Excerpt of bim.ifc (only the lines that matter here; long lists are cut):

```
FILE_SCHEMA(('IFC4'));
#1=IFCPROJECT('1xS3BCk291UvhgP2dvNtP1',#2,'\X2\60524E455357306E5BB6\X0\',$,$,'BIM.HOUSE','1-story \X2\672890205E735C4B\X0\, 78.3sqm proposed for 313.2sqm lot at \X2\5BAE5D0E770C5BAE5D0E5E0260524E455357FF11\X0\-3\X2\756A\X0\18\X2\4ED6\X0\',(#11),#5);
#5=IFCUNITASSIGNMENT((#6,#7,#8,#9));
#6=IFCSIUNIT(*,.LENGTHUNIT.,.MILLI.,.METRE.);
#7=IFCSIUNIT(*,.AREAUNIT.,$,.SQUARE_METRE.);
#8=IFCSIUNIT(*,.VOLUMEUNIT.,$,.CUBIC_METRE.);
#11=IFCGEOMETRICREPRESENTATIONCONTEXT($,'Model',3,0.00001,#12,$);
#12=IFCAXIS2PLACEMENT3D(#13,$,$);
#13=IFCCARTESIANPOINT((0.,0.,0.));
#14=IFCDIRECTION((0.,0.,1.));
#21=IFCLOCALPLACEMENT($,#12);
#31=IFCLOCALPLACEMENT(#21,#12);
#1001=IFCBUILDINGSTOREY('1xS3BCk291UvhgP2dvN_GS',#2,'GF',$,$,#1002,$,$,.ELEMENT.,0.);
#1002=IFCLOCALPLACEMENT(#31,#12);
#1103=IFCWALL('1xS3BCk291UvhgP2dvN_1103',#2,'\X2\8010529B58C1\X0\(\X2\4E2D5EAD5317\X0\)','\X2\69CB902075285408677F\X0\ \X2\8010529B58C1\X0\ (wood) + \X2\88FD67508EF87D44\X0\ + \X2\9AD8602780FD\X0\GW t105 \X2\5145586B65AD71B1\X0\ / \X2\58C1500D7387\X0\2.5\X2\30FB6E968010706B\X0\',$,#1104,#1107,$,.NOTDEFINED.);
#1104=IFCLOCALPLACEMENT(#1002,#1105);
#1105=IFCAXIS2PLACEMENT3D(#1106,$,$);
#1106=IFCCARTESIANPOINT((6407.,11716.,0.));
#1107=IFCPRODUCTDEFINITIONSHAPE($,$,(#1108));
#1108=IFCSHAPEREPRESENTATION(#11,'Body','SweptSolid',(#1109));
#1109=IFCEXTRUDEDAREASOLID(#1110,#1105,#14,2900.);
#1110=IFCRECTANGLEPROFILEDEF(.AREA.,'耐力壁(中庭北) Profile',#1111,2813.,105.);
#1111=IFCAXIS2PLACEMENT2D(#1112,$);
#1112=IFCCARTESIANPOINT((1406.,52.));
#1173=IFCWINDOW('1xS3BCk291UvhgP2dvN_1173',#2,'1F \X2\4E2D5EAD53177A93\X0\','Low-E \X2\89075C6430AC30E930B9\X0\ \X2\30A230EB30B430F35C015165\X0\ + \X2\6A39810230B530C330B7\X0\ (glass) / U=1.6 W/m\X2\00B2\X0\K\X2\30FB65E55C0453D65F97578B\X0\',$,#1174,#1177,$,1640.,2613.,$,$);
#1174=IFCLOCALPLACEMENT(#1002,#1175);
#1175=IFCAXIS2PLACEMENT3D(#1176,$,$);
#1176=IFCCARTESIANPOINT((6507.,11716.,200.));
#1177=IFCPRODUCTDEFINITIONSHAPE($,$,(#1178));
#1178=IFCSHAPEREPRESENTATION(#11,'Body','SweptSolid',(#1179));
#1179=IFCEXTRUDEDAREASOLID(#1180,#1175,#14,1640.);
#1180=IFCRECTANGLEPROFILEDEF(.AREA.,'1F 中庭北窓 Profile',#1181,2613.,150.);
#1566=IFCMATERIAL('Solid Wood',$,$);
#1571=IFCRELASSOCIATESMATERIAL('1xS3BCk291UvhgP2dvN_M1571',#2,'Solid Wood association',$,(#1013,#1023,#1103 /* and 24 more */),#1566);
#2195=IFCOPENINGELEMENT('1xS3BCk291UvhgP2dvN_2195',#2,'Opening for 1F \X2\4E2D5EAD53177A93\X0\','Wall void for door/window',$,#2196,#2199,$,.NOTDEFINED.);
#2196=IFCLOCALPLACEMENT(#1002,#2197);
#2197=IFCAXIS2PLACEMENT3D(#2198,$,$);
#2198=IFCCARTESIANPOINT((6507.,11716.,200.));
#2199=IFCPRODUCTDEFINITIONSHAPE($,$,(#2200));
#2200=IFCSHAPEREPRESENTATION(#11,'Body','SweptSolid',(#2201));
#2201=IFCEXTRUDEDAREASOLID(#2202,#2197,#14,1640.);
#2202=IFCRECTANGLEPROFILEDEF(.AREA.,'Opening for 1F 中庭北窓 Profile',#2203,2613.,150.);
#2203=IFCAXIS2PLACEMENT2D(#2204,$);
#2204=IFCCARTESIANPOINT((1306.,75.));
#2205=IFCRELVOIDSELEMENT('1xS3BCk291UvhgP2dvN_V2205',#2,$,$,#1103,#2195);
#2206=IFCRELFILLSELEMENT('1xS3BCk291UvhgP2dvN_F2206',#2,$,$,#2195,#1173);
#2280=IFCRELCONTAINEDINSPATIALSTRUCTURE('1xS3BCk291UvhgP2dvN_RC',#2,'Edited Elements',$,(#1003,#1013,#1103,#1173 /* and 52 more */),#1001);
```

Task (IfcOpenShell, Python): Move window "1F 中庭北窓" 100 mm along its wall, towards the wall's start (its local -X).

```python
import ifcopenshell
import ifcopenshell.api.geometry
import ifcopenshell.util.placement

model = ifcopenshell.open("bim.ifc")

window = model.by_id(1173)
opening = window.FillsVoids[0].RelatingOpeningElement
wall = opening.VoidsElements[0].RelatingBuildingElement

wall_matrix = ifcopenshell.util.placement.get_local_placement(wall.ObjectPlacement)
shift = wall_matrix[:3, 0] * -100.0
before = ifcopenshell.util.placement.get_local_placement(window.ObjectPlacement)[:3, 3].copy()

# The window is not placed relative to its opening, so move both.
for product in (opening, window):
    matrix = ifcopenshell.util.placement.get_local_placement(product.ObjectPlacement)
    matrix[:3, 3] += shift
    ifcopenshell.api.geometry.edit_object_placement(model, product=product, matrix=matrix, is_si=False)

after = ifcopenshell.util.placement.get_local_placement(window.ObjectPlacement)[:3, 3]
print("window moved by", (after - before).round(3) + 0.0)

model.write("bim_rev.ifc")
```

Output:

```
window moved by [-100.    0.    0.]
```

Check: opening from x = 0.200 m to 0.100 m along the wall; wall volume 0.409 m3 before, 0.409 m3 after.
